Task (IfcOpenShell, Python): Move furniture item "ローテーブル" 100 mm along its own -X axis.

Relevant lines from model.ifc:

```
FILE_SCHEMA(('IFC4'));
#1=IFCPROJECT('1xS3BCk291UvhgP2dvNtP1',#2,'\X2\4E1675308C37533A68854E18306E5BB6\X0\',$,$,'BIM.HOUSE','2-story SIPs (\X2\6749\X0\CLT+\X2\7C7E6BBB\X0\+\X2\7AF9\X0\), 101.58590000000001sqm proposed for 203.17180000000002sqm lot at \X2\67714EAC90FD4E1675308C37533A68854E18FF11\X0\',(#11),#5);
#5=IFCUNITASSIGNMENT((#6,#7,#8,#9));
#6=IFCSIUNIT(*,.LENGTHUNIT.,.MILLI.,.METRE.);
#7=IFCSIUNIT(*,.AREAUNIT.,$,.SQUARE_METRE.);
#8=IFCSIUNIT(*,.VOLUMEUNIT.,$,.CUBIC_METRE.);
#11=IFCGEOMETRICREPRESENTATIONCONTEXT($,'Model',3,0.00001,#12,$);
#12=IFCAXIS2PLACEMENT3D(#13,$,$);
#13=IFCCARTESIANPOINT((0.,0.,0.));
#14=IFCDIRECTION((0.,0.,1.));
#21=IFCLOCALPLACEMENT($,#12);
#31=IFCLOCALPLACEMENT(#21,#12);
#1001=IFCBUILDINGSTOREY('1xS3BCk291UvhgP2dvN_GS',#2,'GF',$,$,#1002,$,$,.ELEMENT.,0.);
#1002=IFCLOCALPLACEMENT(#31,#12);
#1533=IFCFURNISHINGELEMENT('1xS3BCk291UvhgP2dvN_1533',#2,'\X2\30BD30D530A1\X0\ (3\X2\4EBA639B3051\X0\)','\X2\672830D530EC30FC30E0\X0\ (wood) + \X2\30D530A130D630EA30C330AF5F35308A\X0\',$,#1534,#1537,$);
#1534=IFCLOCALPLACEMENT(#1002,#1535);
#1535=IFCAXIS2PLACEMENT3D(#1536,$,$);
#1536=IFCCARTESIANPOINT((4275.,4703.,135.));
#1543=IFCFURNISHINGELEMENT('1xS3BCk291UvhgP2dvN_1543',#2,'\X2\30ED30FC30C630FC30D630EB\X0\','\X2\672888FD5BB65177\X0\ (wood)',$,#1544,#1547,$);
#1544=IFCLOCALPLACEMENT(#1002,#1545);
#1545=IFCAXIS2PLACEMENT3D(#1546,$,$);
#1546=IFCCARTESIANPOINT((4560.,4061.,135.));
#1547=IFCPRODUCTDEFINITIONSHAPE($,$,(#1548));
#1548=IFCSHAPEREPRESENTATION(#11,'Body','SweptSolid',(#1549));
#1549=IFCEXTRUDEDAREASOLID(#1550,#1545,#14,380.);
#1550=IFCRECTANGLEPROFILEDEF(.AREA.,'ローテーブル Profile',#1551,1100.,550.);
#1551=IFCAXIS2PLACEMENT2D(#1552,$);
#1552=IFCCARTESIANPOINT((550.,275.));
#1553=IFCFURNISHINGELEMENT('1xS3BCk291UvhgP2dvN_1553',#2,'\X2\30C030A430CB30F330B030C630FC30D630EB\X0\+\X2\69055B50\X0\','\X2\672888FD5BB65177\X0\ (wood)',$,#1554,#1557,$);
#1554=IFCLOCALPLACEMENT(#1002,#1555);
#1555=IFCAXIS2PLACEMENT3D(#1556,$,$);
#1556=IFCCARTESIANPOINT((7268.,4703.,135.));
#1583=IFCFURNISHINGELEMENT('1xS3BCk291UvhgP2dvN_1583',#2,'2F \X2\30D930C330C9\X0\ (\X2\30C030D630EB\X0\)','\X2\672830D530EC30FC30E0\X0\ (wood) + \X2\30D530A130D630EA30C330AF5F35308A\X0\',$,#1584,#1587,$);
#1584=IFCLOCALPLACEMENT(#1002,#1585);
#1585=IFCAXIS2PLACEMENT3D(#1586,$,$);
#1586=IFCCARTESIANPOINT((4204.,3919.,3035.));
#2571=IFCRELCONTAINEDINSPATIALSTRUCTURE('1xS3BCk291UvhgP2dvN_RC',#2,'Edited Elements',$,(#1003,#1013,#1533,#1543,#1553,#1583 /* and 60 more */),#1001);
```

```python
import ifcopenshell
import ifcopenshell.api.geometry
import ifcopenshell.util.placement

model = ifcopenshell.open("model.ifc")

item = model.by_guid("1xS3BCk291UvhgP2dvN_1543")
matrix = ifcopenshell.util.placement.get_local_placement(item.ObjectPlacement)
matrix[:3, 3] -= matrix[:3, 0] * 100.0
ifcopenshell.api.geometry.edit_object_placement(model, product=item, matrix=matrix, is_si=False)

print(ifcopenshell.util.placement.get_local_placement(item.ObjectPlacement).round(3) + 0.0)

model.write("model_rev.ifc")
```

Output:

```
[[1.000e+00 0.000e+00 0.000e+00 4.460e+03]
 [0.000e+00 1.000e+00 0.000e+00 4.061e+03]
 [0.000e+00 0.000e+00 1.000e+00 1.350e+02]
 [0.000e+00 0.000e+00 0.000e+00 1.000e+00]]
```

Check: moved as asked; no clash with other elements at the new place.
